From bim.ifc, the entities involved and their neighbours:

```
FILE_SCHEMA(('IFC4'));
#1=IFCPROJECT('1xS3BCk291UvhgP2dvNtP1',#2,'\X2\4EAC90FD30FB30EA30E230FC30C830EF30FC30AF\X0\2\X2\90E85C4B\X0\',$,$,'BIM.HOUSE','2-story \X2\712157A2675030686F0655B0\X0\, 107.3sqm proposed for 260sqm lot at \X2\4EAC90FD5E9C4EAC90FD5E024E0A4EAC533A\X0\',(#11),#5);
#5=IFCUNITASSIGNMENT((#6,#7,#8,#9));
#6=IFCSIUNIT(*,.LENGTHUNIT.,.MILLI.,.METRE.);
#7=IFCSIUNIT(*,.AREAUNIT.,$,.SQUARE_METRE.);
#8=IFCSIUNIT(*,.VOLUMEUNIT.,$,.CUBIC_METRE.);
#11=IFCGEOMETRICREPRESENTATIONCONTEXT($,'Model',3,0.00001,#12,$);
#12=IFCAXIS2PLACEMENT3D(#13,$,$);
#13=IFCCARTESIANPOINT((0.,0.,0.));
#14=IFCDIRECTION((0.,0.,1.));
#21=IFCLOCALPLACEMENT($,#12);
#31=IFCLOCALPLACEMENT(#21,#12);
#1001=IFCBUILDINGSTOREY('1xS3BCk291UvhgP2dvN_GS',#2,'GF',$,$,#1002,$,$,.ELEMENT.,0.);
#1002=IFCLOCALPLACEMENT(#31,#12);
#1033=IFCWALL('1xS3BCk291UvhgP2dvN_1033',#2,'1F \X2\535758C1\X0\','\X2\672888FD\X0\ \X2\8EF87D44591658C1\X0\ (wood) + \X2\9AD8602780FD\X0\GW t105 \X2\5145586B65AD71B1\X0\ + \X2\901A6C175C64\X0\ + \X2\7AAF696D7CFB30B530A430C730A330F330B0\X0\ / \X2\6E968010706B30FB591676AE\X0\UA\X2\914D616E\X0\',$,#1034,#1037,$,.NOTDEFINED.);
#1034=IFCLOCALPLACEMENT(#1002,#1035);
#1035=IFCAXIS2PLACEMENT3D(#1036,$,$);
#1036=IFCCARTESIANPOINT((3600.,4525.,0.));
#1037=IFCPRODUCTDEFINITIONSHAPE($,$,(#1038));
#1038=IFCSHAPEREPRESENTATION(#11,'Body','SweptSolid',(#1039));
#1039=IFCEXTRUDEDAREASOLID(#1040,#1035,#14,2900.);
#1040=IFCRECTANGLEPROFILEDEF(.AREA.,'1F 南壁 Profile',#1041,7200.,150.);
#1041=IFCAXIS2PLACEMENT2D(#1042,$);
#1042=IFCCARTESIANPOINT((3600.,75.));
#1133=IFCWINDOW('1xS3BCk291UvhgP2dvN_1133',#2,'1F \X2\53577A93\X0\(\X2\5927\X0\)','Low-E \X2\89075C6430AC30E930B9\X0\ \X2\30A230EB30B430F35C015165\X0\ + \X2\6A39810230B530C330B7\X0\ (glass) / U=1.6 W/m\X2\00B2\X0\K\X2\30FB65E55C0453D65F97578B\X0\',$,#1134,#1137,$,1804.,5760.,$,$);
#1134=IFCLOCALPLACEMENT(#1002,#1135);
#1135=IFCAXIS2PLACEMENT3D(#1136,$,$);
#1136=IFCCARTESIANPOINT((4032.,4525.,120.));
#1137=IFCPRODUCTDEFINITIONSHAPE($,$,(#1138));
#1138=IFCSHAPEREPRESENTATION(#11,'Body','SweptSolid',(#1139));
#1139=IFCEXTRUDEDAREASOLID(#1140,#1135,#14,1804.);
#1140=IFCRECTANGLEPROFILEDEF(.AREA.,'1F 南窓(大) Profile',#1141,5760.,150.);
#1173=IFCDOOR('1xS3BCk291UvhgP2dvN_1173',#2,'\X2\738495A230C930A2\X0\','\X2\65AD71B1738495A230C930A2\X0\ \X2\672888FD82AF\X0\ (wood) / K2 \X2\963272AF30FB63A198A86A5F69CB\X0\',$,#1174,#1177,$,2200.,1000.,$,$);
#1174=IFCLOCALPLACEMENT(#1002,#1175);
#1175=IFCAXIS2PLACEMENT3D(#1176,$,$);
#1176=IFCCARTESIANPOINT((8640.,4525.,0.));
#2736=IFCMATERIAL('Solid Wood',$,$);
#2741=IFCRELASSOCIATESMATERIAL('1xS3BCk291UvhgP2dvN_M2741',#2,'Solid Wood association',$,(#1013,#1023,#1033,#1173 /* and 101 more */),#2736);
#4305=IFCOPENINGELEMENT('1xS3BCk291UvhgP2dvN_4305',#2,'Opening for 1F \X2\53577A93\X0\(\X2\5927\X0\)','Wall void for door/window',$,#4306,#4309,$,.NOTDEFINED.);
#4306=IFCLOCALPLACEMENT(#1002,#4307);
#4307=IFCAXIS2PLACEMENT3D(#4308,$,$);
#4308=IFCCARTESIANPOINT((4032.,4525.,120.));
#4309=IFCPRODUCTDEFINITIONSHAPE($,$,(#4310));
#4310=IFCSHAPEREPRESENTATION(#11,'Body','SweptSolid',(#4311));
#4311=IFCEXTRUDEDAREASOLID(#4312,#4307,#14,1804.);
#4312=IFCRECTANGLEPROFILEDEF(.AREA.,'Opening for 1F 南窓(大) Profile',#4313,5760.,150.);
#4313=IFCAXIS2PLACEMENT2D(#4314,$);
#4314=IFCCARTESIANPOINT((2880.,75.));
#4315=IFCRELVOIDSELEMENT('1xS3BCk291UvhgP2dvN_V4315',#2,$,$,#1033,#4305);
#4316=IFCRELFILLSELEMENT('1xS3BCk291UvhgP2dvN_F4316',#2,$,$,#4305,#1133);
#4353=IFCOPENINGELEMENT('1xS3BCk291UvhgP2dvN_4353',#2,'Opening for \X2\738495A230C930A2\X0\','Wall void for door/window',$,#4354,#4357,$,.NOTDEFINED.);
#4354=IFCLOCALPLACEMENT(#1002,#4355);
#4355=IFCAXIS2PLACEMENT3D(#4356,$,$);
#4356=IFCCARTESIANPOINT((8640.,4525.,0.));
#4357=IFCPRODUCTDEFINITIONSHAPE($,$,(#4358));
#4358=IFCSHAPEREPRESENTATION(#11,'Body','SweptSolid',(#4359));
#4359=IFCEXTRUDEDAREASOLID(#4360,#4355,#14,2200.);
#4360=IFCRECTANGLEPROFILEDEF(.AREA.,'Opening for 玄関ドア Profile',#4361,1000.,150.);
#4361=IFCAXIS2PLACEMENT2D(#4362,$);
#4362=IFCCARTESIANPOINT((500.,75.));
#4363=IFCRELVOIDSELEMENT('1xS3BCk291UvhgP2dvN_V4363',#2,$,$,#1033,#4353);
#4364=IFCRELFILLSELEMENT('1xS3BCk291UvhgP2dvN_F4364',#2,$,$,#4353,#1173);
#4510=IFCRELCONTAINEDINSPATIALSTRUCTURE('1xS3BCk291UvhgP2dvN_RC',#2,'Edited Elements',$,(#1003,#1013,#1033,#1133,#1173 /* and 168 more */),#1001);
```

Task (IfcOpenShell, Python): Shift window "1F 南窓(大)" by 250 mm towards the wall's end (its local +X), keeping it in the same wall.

```python
import ifcopenshell
import ifcopenshell.api.geometry
import ifcopenshell.util.placement
import ifcopenshell.util.unit

model = ifcopenshell.open("bim.ifc")
unit_scale = ifcopenshell.util.unit.calculate_unit_scale(model)

window = model.by_id(1133)
opening = window.FillsVoids[0].RelatingOpeningElement
wall = opening.VoidsElements[0].RelatingBuildingElement

wall_matrix = ifcopenshell.util.placement.get_local_placement(wall.ObjectPlacement)
shift = wall_matrix[:3, 0] * 0.25 / unit_scale
before = ifcopenshell.util.placement.get_local_placement(window.ObjectPlacement)[:3, 3].copy()

# The window is not placed relative to its opening, so move both.
for product in (opening, window):
    matrix = ifcopenshell.util.placement.get_local_placement(product.ObjectPlacement)
    matrix[:3, 3] += shift
    ifcopenshell.api.geometry.edit_object_placement(model, product=product, matrix=matrix, is_si=False)

after = ifcopenshell.util.placement.get_local_placement(window.ObjectPlacement)[:3, 3]
print("window moved by", (after - before).round(3) + 0.0)

model.write("bim-out.ifc")
```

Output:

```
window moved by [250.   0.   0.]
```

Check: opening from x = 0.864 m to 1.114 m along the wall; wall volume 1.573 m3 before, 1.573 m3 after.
